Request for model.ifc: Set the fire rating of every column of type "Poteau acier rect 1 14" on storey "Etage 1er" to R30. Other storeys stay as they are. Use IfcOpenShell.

First a look at what the model holds.

```python
import ifcopenshell
import ifcopenshell.util.element

model = ifcopenshell.open("model.ifc")
print(model.schema)
storey = next(s for s in model.by_type("IfcBuildingStorey") if s.Name == "Etage 1er")
columns = [e for e in ifcopenshell.util.element.get_decomposition(storey) if e.is_a("IfcColumn")]
seen = {}
for e in columns:
    element_type = ifcopenshell.util.element.get_type(e)
    key = (element_type.Name if element_type != e and element_type else None, ifcopenshell.util.element.get_pset(e, "Pset_ColumnCommon", "FireRating"))
    seen[key] = seen.get(key, 0) + 1
for (name, value), count in sorted(seen.items(), key=str):
    print(count, "x", name, "|", value)
```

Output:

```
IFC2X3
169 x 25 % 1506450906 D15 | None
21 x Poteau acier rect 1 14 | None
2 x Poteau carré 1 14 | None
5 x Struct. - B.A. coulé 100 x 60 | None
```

```python
import ifcopenshell
import ifcopenshell.api.pset
import ifcopenshell.util.element

model = ifcopenshell.open("model.ifc")

storey = next(s for s in model.by_type("IfcBuildingStorey") if s.Name == "Etage 1er")
columns = [e for e in ifcopenshell.util.element.get_decomposition(storey) if e.is_a("IfcColumn")]

count = 0
for e in columns:
    element_type = ifcopenshell.util.element.get_type(e)
    if element_type in (None, e) or element_type.Name != "Poteau acier rect 1 14":
        continue
    # add_pset returns the element's existing set when there is one.
    pset = ifcopenshell.api.pset.add_pset(model, product=e, name="Pset_ColumnCommon")
    ifcopenshell.api.pset.edit_pset(model, pset=pset, properties={"FireRating": "R30"})
    count += 1

print(count, "columns updated")

model.write("model_v2.ifc")
```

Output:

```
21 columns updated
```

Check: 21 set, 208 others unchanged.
